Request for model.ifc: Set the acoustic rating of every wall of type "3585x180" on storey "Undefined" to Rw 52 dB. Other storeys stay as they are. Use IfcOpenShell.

First a look at what the model holds.

```python
import ifcopenshell
import ifcopenshell.util.element

model = ifcopenshell.open("model.ifc")
print(model.schema)
storey = next(s for s in model.by_type("IfcBuildingStorey") if s.Name == "Undefined")
walls = [e for e in ifcopenshell.util.element.get_decomposition(storey) if e.is_a("IfcWall")]
seen = {}
for e in walls:
    element_type = ifcopenshell.util.element.get_type(e)
    key = (element_type.Name if element_type != e and element_type else None, ifcopenshell.util.element.get_pset(e, "Pset_WallCommon", "AcousticRating"))
    seen[key] = seen.get(key, 0) + 1
for (name, value), count in sorted(seen.items(), key=str):
    print(count, "x", name, "|", value)
```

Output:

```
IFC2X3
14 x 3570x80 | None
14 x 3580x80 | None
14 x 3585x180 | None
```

```python
import ifcopenshell
import ifcopenshell.api.pset
import ifcopenshell.util.element

model = ifcopenshell.open("model.ifc")

storey = next(s for s in model.by_type("IfcBuildingStorey") if s.Name == "Undefined")
walls = [e for e in ifcopenshell.util.element.get_decomposition(storey) if e.is_a("IfcWall")]

count = 0
for e in walls:
    element_type = ifcopenshell.util.element.get_type(e)
    if element_type in (None, e) or element_type.Name != "3585x180":
        continue
    found = ifcopenshell.util.element.get_pset(e, "Pset_WallCommon", should_inherit=False)
    if found:
        pset = model.by_id(found["id"])
        if len(ifcopenshell.util.element.get_elements_by_pset(pset)) > 1:
            pset = ifcopenshell.api.pset.unshare_pset(model, products=[e], pset=pset)[0]
    else:
        pset = ifcopenshell.api.pset.add_pset(model, product=e, name="Pset_WallCommon")
    ifcopenshell.api.pset.edit_pset(model, pset=pset, properties={"AcousticRating": "Rw 52 dB"})
    count += 1

print(count, "walls updated")

model.write("model_edited.ifc")
```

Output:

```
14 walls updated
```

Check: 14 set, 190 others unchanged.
